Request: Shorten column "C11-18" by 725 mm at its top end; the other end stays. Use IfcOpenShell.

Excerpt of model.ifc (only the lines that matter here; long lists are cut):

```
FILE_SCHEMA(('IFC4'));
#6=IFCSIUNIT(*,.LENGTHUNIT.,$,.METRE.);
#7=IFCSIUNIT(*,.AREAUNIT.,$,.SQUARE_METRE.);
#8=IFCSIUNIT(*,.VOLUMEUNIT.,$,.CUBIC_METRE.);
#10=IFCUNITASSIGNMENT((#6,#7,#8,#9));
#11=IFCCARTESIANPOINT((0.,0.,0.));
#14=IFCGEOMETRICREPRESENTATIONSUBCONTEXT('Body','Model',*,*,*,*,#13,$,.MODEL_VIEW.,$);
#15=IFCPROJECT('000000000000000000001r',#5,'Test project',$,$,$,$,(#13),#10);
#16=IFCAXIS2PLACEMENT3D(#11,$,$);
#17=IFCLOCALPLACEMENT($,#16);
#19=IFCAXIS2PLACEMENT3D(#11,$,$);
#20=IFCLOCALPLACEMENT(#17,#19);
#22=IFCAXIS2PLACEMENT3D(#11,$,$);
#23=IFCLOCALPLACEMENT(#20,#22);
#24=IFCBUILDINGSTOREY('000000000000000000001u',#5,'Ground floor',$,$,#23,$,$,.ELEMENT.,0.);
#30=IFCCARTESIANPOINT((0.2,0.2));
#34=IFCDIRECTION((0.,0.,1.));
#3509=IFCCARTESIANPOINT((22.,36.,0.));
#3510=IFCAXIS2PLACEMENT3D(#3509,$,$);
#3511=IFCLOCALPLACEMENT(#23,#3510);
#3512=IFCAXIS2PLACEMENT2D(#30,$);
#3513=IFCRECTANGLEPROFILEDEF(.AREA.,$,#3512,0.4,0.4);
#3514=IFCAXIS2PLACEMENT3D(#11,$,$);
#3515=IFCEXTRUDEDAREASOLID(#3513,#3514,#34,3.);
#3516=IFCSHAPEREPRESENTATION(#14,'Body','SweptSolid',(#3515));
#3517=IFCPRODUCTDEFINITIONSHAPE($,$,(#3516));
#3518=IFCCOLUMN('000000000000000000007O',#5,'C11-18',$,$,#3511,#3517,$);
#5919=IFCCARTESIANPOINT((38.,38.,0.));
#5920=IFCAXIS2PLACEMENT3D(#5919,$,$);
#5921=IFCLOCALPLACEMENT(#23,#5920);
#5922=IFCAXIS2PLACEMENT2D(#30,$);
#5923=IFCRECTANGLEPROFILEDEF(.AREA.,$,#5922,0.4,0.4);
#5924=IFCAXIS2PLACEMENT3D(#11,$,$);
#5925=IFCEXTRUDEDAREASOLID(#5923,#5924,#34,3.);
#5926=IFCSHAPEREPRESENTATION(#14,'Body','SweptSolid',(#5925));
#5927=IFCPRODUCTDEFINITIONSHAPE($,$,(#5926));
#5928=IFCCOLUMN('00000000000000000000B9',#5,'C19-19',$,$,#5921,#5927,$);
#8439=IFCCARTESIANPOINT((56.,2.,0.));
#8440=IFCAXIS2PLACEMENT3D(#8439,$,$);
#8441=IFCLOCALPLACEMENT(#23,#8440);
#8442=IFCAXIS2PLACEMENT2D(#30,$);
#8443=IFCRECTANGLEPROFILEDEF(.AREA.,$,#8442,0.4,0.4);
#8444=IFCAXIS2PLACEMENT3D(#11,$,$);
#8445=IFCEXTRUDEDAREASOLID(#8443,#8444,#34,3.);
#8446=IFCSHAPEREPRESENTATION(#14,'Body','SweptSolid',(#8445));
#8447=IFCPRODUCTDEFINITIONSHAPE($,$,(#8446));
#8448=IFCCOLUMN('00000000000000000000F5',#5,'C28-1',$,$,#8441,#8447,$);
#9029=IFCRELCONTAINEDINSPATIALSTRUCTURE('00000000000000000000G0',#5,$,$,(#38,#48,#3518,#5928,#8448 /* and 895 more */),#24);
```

```python
import ifcopenshell
import ifcopenshell.util.representation
import ifcopenshell.util.unit

model = ifcopenshell.open("model.ifc")
unit_scale = ifcopenshell.util.unit.calculate_unit_scale(model)

member = model.by_id(3518)
change = -0.725 / unit_scale

# The extrusion runs towards the end named, so only its depth changes.
body = ifcopenshell.util.representation.get_representation(member, "Model", "Body")
solid = body.Items[0]
old_length = solid.Depth
solid.Depth += change

print(f"length {old_length:g} -> {solid.Depth:g}")

model.write("model-out.ifc")
```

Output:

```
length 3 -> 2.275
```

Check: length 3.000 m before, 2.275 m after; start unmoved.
